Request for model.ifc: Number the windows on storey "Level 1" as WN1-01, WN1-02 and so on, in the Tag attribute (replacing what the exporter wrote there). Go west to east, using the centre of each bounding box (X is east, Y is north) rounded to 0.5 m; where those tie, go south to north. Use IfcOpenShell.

First a look at what the model holds.

```python
import ifcopenshell
import ifcopenshell.util.element
import ifcopenshell.util.placement

model = ifcopenshell.open("model.ifc")
print(model.schema)
storey = next(s for s in model.by_type("IfcBuildingStorey") if s.Name == "Level 1")
windows = [e for e in ifcopenshell.util.element.get_decomposition(storey) if e.is_a("IfcWindow")]
for e in sorted(windows, key=lambda e: e.id()):
    origin = ifcopenshell.util.placement.get_local_placement(e.ObjectPlacement)[:3, 3]
    print(e.id(), e.Tag, e.Name, origin.round(2) + 0.0, sep=" | ")
```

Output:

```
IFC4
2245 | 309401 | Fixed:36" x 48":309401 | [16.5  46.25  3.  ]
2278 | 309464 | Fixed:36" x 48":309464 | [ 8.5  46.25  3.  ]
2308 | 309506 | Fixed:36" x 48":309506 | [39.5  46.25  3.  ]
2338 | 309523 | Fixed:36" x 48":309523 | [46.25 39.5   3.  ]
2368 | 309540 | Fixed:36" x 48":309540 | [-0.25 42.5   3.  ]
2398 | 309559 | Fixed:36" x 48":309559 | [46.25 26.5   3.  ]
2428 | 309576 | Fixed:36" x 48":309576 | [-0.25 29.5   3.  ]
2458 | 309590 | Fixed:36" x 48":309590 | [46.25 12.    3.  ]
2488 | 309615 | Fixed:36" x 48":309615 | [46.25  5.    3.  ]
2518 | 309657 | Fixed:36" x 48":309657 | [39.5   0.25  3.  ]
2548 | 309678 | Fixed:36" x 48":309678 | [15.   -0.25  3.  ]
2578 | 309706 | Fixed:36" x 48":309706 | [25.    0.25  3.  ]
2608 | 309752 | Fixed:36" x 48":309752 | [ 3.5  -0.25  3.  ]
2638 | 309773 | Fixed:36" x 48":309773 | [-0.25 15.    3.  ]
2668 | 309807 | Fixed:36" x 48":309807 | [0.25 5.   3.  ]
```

```python
import ifcopenshell
import ifcopenshell.geom
import ifcopenshell.util.element
import ifcopenshell.util.shape

model = ifcopenshell.open("model.ifc")
settings = ifcopenshell.geom.settings()
settings.set("use-world-coords", True)


def centre(element):
    shape = ifcopenshell.geom.create_shape(settings, element)
    return ifcopenshell.util.shape.get_bbox_centroid(shape.geometry)


storey = next(s for s in model.by_type("IfcBuildingStorey") if s.Name == "Level 1")
windows = [e for e in ifcopenshell.util.element.get_decomposition(storey) if e.is_a("IfcWindow")]

# Insertion points can sit at a corner or the storey origin, so sort by the geometry (in metres).
centres = {e: centre(e) for e in windows}
windows.sort(key=lambda e: (round(centres[e][0] / 0.5), centres[e][1]))

for i, e in enumerate(windows, start=1):
    number = f"WN1-{i:02d}"
    e.Tag = number
    print(e.id(), number)

model.write("model_updated.ifc")
```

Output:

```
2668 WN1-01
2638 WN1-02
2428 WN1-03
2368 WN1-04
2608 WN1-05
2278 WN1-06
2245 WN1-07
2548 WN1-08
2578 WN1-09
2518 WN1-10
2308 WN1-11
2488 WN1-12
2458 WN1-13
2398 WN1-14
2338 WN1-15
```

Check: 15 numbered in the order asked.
